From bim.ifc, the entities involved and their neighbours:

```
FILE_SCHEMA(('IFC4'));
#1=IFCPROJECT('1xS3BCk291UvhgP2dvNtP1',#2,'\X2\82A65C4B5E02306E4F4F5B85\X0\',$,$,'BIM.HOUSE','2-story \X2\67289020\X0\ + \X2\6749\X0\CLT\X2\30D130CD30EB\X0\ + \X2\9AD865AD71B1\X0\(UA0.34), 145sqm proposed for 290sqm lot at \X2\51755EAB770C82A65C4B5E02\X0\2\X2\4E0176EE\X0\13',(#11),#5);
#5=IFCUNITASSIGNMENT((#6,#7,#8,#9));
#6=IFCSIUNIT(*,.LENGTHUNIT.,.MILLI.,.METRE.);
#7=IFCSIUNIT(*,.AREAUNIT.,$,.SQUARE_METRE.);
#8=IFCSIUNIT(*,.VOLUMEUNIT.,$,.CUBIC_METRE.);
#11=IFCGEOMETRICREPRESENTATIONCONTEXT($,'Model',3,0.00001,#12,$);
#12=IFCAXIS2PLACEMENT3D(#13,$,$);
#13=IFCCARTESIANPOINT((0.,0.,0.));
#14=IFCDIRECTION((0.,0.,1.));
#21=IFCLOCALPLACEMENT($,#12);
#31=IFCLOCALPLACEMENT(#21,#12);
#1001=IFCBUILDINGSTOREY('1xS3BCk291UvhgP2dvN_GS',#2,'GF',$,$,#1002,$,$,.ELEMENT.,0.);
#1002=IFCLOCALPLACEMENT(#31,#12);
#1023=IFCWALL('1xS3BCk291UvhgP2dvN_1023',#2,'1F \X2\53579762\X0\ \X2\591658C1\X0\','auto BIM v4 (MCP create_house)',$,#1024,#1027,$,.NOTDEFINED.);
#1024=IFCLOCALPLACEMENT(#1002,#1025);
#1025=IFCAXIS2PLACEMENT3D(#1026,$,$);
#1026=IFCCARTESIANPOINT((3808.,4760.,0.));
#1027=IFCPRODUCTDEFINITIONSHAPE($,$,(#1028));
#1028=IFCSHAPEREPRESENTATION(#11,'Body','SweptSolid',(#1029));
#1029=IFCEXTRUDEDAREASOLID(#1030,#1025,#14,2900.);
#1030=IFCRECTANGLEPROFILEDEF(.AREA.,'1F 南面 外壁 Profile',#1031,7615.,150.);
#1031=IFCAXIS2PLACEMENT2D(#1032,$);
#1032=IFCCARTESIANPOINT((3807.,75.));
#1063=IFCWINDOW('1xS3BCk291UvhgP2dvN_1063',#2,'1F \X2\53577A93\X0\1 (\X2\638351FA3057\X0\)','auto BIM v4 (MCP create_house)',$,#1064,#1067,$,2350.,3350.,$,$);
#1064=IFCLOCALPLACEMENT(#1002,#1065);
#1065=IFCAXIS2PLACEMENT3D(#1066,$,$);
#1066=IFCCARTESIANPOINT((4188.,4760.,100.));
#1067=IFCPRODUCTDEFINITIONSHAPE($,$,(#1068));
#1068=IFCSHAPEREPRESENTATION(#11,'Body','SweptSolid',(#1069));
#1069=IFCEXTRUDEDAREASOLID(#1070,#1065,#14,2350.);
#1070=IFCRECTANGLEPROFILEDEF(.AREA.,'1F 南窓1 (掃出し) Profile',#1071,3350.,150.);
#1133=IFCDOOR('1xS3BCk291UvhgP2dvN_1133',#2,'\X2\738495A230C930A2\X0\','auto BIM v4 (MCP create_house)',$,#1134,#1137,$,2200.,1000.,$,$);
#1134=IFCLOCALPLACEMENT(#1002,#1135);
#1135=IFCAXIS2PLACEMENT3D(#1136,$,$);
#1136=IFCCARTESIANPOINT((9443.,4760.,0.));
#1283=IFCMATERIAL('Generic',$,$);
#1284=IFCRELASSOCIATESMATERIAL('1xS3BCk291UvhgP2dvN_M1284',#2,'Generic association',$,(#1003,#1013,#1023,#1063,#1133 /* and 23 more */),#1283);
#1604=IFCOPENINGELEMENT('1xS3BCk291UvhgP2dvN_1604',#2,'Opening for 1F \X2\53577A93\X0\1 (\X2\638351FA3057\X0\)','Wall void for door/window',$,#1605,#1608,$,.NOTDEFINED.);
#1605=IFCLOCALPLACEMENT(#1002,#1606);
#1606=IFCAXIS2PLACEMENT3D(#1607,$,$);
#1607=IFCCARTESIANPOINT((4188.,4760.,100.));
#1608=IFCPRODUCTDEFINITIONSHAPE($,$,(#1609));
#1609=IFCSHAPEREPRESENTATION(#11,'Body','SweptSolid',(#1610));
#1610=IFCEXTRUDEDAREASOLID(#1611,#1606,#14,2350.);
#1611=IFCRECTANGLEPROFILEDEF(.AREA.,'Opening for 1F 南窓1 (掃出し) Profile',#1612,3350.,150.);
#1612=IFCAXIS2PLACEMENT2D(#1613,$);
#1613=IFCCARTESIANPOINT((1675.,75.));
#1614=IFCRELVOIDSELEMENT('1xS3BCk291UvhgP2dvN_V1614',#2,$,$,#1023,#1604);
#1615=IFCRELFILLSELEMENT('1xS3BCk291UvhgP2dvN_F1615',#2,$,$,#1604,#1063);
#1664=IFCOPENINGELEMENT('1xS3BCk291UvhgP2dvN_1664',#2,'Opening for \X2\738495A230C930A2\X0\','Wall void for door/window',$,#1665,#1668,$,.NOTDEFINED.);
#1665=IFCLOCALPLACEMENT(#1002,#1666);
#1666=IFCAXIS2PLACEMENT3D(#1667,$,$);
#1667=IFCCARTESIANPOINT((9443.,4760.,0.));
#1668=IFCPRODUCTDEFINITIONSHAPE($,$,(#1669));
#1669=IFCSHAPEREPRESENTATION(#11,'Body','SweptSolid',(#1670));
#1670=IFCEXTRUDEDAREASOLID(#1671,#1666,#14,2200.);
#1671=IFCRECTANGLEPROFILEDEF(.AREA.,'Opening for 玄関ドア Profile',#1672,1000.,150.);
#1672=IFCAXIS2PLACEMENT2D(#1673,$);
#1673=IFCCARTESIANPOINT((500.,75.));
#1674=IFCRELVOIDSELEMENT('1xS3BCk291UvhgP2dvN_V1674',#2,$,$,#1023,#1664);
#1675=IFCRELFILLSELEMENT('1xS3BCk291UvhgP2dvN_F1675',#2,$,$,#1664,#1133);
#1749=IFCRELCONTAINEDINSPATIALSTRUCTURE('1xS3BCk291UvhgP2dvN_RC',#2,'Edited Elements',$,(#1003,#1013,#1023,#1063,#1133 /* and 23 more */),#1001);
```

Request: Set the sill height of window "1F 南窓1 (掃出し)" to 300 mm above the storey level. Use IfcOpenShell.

```python
import numpy as np
import ifcopenshell
import ifcopenshell.api.geometry
import ifcopenshell.geom
import ifcopenshell.util.element
import ifcopenshell.util.placement
import ifcopenshell.util.shape
import ifcopenshell.util.unit

model = ifcopenshell.open("bim.ifc")
unit_scale = ifcopenshell.util.unit.calculate_unit_scale(model)

window = model.by_guid("1xS3BCk291UvhgP2dvN_1063")
opening = window.FillsVoids[0].RelatingOpeningElement
storey = ifcopenshell.util.element.get_container(window, ifc_class="IfcBuildingStorey")
level = ifcopenshell.util.placement.get_local_placement(storey.ObjectPlacement)[2, 3]

# The opening's origin need not be at the sill, so measure its lowest point.
shape = ifcopenshell.geom.create_shape(ifcopenshell.geom.settings(), opening)
bottom = ifcopenshell.util.shape.get_shape_bottom_elevation(shape, shape.geometry) / unit_scale
dz = level + 300.0 - bottom

shift = np.array([0.0, 0.0, dz])
# The window is not placed relative to its opening, so move both.
for product in (opening, window):
    matrix = ifcopenshell.util.placement.get_local_placement(product.ObjectPlacement)
    matrix[:3, 3] += shift
    ifcopenshell.api.geometry.edit_object_placement(model, product=product, matrix=matrix, is_si=False)

print(f"moved by {dz * unit_scale:+.3f} m")

model.write("bim_v2.ifc")
```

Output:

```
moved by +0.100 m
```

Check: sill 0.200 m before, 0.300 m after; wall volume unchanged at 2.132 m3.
